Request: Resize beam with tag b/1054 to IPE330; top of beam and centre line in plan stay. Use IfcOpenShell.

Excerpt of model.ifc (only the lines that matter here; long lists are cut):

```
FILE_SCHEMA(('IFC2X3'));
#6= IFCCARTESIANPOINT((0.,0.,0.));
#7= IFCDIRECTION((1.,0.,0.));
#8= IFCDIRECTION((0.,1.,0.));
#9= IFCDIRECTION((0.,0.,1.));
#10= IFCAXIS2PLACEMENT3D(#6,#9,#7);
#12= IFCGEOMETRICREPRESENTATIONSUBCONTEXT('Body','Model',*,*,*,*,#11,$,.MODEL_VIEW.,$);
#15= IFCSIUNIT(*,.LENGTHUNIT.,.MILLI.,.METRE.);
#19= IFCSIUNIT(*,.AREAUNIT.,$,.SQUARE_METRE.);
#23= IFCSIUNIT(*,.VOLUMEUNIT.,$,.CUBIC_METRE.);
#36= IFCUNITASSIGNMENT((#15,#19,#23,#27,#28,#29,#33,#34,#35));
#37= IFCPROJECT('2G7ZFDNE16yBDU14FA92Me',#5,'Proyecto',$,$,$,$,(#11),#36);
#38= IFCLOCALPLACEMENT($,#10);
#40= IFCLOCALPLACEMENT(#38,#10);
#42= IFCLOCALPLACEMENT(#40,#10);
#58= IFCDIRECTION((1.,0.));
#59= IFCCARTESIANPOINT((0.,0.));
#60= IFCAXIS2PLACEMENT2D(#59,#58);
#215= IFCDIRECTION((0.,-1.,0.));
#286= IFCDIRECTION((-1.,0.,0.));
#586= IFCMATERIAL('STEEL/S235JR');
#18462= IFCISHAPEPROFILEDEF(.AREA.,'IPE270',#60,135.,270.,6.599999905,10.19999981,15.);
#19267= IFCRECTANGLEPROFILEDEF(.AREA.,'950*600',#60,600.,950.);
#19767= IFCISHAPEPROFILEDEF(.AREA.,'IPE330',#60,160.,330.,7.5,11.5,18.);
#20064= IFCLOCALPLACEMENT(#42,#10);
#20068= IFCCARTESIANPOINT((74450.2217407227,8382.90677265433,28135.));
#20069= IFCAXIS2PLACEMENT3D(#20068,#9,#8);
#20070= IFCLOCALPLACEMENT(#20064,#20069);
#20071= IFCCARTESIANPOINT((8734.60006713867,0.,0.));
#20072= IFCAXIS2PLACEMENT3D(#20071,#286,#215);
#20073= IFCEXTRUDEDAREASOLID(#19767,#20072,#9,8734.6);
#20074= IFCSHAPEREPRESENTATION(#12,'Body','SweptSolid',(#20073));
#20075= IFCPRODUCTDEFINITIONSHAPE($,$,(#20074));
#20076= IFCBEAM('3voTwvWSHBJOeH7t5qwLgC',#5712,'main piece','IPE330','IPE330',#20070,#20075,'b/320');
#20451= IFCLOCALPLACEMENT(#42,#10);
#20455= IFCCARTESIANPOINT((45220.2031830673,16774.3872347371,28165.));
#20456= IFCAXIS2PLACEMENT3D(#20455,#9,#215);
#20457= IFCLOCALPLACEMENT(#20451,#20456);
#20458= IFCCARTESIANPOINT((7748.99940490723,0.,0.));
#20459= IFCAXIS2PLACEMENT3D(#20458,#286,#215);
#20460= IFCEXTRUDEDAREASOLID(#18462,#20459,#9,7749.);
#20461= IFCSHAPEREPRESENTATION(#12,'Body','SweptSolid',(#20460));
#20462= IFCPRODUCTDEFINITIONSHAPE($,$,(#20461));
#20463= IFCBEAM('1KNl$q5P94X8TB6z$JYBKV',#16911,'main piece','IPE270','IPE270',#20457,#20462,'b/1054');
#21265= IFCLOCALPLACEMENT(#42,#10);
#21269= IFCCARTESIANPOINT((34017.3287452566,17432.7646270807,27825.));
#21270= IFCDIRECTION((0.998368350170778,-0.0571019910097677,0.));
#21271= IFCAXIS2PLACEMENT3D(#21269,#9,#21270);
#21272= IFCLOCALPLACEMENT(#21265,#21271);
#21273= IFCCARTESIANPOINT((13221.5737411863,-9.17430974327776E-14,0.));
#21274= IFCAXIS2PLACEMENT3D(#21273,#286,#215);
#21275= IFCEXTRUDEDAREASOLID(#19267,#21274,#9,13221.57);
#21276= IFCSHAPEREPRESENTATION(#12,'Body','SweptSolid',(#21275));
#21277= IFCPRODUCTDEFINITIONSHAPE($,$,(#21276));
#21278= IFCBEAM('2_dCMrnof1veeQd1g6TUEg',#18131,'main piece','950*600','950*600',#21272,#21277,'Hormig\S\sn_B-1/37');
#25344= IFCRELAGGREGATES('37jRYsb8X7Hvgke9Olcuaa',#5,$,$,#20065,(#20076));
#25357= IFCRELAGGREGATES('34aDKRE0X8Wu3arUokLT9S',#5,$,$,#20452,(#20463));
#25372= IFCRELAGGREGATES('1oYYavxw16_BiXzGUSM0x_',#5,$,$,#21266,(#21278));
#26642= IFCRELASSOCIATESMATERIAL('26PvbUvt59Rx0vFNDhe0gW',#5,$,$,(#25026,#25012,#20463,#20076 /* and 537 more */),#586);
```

```python
import ifcopenshell
import ifcopenshell.util.element
import ifcopenshell.util.representation

model = ifcopenshell.open("model.ifc")

member = model.by_guid("1KNl$q5P94X8TB6z$JYBKV")
source = next(p for p in model.by_type("IfcIShapeProfileDef") if p.ProfileName == "IPE330")

body = ifcopenshell.util.representation.get_representation(member, "Model", "Body")
solid = body.Items[0]
old_profile = solid.SweptArea

# Copy the section's sizes but keep this member's own profile position.
profile = ifcopenshell.util.element.copy(model, source)
# Profiles are centred, so shift by half the change in depth to hold the top.
shift = (old_profile.OverallDepth - profile.OverallDepth) / 2
x, y = old_profile.Position.Location.Coordinates
up = (0.0, 1.0)  # upwards, in the solid's own plane
location = model.createIfcCartesianPoint((x + up[0] * shift, y + up[1] * shift))
profile.Position = model.createIfcAxis2Placement2D(location, old_profile.Position.RefDirection)
solid.SweptArea = profile
if not model.get_total_inverses(old_profile):
    ifcopenshell.util.element.remove_deep2(model, old_profile)
member.Description = member.Description.replace("IPE270", "IPE330")
member.ObjectType = member.ObjectType.replace("IPE270", "IPE330")

print(solid.SweptArea)

model.write("model_edited.ifc")
```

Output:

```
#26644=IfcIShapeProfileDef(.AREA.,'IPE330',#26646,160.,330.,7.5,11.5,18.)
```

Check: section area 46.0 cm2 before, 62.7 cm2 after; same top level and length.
